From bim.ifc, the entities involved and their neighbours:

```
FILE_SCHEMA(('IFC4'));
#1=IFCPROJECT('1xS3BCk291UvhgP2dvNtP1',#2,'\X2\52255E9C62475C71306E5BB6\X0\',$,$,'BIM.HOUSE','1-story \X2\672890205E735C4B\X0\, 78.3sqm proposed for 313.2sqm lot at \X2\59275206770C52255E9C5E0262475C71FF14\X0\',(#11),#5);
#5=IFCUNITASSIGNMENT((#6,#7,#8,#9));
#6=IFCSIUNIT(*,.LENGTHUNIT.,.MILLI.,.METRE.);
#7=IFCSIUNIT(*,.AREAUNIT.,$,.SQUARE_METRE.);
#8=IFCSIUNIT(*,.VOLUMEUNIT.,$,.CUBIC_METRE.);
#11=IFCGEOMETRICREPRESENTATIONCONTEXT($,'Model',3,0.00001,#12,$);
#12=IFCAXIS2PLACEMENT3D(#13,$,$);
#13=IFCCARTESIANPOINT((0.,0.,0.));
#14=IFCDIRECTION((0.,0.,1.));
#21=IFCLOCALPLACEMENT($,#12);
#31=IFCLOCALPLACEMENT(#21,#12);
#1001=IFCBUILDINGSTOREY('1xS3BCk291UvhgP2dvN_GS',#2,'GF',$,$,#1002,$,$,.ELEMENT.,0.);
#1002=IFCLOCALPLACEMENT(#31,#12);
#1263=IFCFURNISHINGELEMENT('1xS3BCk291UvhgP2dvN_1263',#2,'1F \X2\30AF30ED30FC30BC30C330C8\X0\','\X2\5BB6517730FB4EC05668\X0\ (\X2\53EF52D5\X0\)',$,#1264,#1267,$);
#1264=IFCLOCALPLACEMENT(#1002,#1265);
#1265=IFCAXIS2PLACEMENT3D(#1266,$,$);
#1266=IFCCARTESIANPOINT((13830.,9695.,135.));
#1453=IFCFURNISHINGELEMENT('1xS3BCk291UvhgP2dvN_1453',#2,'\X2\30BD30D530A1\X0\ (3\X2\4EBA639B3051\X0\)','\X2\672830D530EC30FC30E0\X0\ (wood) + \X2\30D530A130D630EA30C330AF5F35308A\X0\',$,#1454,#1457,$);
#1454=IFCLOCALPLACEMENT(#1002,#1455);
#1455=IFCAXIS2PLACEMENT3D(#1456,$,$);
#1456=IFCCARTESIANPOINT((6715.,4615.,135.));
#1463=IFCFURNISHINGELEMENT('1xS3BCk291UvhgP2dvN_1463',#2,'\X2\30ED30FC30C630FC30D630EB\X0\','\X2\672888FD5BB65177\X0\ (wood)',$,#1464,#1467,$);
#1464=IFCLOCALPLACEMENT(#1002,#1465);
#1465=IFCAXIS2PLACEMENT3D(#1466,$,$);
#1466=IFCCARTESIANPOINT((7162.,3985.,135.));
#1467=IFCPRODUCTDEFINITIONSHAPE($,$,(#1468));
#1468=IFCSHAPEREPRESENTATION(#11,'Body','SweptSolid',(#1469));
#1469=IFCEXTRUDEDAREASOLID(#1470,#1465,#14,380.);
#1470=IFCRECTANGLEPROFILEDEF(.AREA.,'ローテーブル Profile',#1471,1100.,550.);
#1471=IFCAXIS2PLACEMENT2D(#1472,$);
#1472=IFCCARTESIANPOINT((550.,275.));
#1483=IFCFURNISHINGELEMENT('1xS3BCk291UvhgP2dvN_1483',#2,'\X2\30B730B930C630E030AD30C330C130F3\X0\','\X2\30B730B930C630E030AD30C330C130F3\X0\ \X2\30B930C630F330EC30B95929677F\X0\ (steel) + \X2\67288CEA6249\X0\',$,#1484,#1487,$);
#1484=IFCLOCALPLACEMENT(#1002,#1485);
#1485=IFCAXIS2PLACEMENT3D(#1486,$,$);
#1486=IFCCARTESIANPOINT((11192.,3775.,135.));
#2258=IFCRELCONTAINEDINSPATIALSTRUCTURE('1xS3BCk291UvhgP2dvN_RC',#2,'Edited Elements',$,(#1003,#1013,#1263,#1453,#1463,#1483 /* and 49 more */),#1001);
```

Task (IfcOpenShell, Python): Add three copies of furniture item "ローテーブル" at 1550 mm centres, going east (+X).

```python
import numpy as np
import ifcopenshell
import ifcopenshell.api.geometry
import ifcopenshell.api.root
import ifcopenshell.util.element
import ifcopenshell.util.placement
import ifcopenshell.util.unit

model = ifcopenshell.open("bim.ifc")
unit_scale = ifcopenshell.util.unit.calculate_unit_scale(model)


def reuse_history(source, copy):
    """copy_class also copies each property set's owner history, people and application; keep the originals."""
    for rel in copy.IsDefinedBy:
        if rel.is_a("IfcRelDefinesByProperties") and (history := rel.RelatingPropertyDefinition.OwnerHistory):
            rel.RelatingPropertyDefinition.OwnerHistory = source.OwnerHistory
            ifcopenshell.util.element.remove_deep2(model, history)


source = model.by_guid("1xS3BCk291UvhgP2dvN_1463")
base = ifcopenshell.util.placement.get_local_placement(source.ObjectPlacement)
step = np.array([1.0, 0.0, 0.0]) * 1.55 / unit_scale

for i in range(1, 4):
    copy = ifcopenshell.api.root.copy_class(model, product=source)
    copy.Representation = ifcopenshell.util.element.copy_deep(
        model, source.Representation, exclude=["IfcGeometricRepresentationContext", "IfcRepresentationMap"]
    )
    reuse_history(source, copy)
    matrix = base.copy()
    matrix[:3, 3] += i * step
    print("added at", matrix[:3, 3].round(3) + 0.0)
    ifcopenshell.api.geometry.edit_object_placement(model, product=copy, matrix=matrix, is_si=False)

model.write("bim-out.ifc")
```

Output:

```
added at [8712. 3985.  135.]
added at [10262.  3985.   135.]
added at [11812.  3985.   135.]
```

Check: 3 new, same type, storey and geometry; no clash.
